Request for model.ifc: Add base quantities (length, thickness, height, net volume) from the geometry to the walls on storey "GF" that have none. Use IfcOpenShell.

First a look at what the model holds.

```python
import ifcopenshell
import ifcopenshell.util.element
import ifcopenshell.util.unit

model = ifcopenshell.open("model.ifc")
print(model.schema)
for unit_type in ("LENGTHUNIT", "AREAUNIT", "VOLUMEUNIT"):
    print(unit_type, ifcopenshell.util.unit.calculate_unit_scale(model, unit_type))
storey = next(s for s in model.by_type("IfcBuildingStorey") if s.Name == "GF")
walls = [e for e in ifcopenshell.util.element.get_decomposition(storey) if e.is_a("IfcWall")]
for e in sorted(walls, key=lambda e: e.id()):
    print(e.id(), e.is_a(), e.Name, list(ifcopenshell.util.element.get_psets(e, qtos_only=True)), sep=" | ")
```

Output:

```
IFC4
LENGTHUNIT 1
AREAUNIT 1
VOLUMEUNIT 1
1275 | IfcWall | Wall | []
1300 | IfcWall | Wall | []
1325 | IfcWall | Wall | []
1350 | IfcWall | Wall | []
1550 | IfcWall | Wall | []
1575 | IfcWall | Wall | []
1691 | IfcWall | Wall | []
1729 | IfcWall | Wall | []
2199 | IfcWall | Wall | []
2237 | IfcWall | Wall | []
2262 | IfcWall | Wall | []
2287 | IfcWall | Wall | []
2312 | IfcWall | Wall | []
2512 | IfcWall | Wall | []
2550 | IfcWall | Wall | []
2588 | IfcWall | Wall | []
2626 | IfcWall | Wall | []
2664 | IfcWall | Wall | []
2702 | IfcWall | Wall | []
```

```python
import ifcopenshell
import ifcopenshell.api.pset
import ifcopenshell.geom
import ifcopenshell.util.element
import ifcopenshell.util.shape
import ifcopenshell.util.unit

model = ifcopenshell.open("model.ifc")
unit_scale = ifcopenshell.util.unit.calculate_unit_scale(model)
volume_scale = ifcopenshell.util.unit.calculate_unit_scale(model, "VOLUMEUNIT")
settings = ifcopenshell.geom.settings()

storey = next(s for s in model.by_type("IfcBuildingStorey") if s.Name == "GF")
walls = [e for e in ifcopenshell.util.element.get_decomposition(storey) if e.is_a("IfcWall")]

for e in sorted(walls, key=lambda e: e.id()):
    if ifcopenshell.util.element.get_psets(e, qtos_only=True, should_inherit=False):
        continue
    # Geometry comes back in metres, in the element's own axes.
    shape = ifcopenshell.geom.create_shape(settings, e)
    values = {
        "Length": ifcopenshell.util.shape.get_x(shape.geometry) / unit_scale,
        "Width": ifcopenshell.util.shape.get_y(shape.geometry) / unit_scale,
        "Height": ifcopenshell.util.shape.get_z(shape.geometry) / unit_scale,
        "NetVolume": ifcopenshell.util.shape.get_volume(shape.geometry) / volume_scale,
    }
    qto = ifcopenshell.api.pset.add_qto(model, product=e, name="Qto_WallBaseQuantities")
    ifcopenshell.api.pset.edit_qto(model, qto=qto, properties=values)
    print(e.id(), {k: round(v, 3) for k, v in values.items()})

model.write("model_v2.ifc")
```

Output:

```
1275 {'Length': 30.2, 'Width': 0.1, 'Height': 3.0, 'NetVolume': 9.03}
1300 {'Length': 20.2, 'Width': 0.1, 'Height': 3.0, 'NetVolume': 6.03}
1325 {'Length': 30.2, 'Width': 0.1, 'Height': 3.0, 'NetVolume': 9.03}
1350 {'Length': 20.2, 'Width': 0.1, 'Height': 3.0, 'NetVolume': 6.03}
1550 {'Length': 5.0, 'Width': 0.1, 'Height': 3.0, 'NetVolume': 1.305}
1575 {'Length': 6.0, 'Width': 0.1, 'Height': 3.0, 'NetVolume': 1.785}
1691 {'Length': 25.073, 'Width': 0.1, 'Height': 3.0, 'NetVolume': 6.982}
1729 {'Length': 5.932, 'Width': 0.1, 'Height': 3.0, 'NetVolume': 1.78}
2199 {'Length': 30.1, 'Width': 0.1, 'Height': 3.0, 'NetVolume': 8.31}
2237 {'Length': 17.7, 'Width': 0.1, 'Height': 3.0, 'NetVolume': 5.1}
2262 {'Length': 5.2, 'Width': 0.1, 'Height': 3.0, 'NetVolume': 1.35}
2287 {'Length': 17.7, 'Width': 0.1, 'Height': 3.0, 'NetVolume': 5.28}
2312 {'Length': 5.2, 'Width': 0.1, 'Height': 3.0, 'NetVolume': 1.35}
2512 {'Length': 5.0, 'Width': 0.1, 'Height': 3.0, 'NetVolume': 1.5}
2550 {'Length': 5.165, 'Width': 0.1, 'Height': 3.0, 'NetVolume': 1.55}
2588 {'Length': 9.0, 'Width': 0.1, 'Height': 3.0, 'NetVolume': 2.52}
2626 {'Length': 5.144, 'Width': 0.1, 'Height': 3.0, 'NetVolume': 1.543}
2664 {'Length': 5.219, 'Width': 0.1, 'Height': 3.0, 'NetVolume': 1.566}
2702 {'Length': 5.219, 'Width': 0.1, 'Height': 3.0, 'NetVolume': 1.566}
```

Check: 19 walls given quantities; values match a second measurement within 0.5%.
